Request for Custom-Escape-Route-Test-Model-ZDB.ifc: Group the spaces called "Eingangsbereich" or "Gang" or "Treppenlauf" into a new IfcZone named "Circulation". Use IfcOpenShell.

First a look at what the model holds.

```python
import ifcopenshell

model = ifcopenshell.open("Custom-Escape-Route-Test-Model-ZDB.ifc")
print(model.schema)
seen = {}
for space in model.by_type("IfcSpace"):
    seen[space.LongName] = seen.get(space.LongName, 0) + 1
for name, count in sorted(seen.items(), key=str):
    print(count, "x", name)
print("zones:", [z.Name for z in model.by_type("IfcZone")][:20])
```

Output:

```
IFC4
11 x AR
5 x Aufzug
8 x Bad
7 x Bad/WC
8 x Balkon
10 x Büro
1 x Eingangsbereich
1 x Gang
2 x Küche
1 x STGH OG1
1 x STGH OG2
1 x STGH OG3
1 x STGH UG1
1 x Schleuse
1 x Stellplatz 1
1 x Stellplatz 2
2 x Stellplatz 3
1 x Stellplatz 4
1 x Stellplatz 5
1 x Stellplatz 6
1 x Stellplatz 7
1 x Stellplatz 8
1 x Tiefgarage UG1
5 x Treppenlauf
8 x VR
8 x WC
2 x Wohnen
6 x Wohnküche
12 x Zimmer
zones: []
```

```python
import ifcopenshell
import ifcopenshell.api.group
import ifcopenshell.api.root

model = ifcopenshell.open("Custom-Escape-Route-Test-Model-ZDB.ifc")

names = {"Eingangsbereich", "Gang", "Treppenlauf"}
spaces = [s for s in model.by_type("IfcSpace") if s.LongName in names]

zone = ifcopenshell.api.root.create_entity(model, ifc_class="IfcZone", name="Circulation")
ifcopenshell.api.group.assign_group(model, products=spaces, group=zone)
print(len(spaces), "spaces in", zone.Name)

model.write("Custom-Escape-Route-Test-Model-ZDB_updated.ifc")
```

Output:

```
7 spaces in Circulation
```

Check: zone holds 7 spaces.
